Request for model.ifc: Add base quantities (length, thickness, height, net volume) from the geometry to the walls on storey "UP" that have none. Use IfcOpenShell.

First a look at what the model holds.

```python
import ifcopenshell
import ifcopenshell.util.element
import ifcopenshell.util.unit

model = ifcopenshell.open("model.ifc")
print(model.schema)
for unit_type in ("LENGTHUNIT", "AREAUNIT", "VOLUMEUNIT"):
    print(unit_type, ifcopenshell.util.unit.calculate_unit_scale(model, unit_type))
storey = next(s for s in model.by_type("IfcBuildingStorey") if s.Name == "UP")
walls = [e for e in ifcopenshell.util.element.get_decomposition(storey) if e.is_a("IfcWall")]
for e in sorted(walls, key=lambda e: e.id()):
    print(e.id(), e.is_a(), e.Name, list(ifcopenshell.util.element.get_psets(e, qtos_only=True)), sep=" | ")
```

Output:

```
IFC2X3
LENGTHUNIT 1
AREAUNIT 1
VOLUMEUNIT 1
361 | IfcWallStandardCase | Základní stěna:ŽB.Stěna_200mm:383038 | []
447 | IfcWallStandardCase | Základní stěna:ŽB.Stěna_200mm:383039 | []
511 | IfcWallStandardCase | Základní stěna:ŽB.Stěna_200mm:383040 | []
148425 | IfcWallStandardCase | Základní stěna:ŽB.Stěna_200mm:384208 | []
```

```python
import ifcopenshell
import ifcopenshell.api.pset
import ifcopenshell.geom
import ifcopenshell.util.element
import ifcopenshell.util.shape
import ifcopenshell.util.unit

model = ifcopenshell.open("model.ifc")
unit_scale = ifcopenshell.util.unit.calculate_unit_scale(model)
volume_scale = ifcopenshell.util.unit.calculate_unit_scale(model, "VOLUMEUNIT")
settings = ifcopenshell.geom.settings()

storey = next(s for s in model.by_type("IfcBuildingStorey") if s.Name == "UP")
walls = [e for e in ifcopenshell.util.element.get_decomposition(storey) if e.is_a("IfcWall")]

for e in sorted(walls, key=lambda e: e.id()):
    if ifcopenshell.util.element.get_psets(e, qtos_only=True, should_inherit=False):
        continue
    # Geometry comes back in metres, in the element's own axes.
    shape = ifcopenshell.geom.create_shape(settings, e)
    values = {
        "Length": ifcopenshell.util.shape.get_x(shape.geometry) / unit_scale,
        "Width": ifcopenshell.util.shape.get_y(shape.geometry) / unit_scale,
        "Height": ifcopenshell.util.shape.get_z(shape.geometry) / unit_scale,
        "NetVolume": ifcopenshell.util.shape.get_volume(shape.geometry) / volume_scale,
    }
    qto = ifcopenshell.api.pset.add_qto(model, product=e, name="BaseQuantities")
    ifcopenshell.api.pset.edit_qto(model, qto=qto, properties=values)
    print(e.id(), {k: round(v, 3) for k, v in values.items()})

model.write("model_edited.ifc")
```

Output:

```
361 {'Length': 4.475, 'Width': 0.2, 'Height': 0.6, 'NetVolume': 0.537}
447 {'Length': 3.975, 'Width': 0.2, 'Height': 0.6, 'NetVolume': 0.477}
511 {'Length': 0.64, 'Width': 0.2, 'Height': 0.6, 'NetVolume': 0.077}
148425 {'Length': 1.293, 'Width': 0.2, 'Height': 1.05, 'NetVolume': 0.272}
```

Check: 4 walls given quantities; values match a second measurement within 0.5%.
